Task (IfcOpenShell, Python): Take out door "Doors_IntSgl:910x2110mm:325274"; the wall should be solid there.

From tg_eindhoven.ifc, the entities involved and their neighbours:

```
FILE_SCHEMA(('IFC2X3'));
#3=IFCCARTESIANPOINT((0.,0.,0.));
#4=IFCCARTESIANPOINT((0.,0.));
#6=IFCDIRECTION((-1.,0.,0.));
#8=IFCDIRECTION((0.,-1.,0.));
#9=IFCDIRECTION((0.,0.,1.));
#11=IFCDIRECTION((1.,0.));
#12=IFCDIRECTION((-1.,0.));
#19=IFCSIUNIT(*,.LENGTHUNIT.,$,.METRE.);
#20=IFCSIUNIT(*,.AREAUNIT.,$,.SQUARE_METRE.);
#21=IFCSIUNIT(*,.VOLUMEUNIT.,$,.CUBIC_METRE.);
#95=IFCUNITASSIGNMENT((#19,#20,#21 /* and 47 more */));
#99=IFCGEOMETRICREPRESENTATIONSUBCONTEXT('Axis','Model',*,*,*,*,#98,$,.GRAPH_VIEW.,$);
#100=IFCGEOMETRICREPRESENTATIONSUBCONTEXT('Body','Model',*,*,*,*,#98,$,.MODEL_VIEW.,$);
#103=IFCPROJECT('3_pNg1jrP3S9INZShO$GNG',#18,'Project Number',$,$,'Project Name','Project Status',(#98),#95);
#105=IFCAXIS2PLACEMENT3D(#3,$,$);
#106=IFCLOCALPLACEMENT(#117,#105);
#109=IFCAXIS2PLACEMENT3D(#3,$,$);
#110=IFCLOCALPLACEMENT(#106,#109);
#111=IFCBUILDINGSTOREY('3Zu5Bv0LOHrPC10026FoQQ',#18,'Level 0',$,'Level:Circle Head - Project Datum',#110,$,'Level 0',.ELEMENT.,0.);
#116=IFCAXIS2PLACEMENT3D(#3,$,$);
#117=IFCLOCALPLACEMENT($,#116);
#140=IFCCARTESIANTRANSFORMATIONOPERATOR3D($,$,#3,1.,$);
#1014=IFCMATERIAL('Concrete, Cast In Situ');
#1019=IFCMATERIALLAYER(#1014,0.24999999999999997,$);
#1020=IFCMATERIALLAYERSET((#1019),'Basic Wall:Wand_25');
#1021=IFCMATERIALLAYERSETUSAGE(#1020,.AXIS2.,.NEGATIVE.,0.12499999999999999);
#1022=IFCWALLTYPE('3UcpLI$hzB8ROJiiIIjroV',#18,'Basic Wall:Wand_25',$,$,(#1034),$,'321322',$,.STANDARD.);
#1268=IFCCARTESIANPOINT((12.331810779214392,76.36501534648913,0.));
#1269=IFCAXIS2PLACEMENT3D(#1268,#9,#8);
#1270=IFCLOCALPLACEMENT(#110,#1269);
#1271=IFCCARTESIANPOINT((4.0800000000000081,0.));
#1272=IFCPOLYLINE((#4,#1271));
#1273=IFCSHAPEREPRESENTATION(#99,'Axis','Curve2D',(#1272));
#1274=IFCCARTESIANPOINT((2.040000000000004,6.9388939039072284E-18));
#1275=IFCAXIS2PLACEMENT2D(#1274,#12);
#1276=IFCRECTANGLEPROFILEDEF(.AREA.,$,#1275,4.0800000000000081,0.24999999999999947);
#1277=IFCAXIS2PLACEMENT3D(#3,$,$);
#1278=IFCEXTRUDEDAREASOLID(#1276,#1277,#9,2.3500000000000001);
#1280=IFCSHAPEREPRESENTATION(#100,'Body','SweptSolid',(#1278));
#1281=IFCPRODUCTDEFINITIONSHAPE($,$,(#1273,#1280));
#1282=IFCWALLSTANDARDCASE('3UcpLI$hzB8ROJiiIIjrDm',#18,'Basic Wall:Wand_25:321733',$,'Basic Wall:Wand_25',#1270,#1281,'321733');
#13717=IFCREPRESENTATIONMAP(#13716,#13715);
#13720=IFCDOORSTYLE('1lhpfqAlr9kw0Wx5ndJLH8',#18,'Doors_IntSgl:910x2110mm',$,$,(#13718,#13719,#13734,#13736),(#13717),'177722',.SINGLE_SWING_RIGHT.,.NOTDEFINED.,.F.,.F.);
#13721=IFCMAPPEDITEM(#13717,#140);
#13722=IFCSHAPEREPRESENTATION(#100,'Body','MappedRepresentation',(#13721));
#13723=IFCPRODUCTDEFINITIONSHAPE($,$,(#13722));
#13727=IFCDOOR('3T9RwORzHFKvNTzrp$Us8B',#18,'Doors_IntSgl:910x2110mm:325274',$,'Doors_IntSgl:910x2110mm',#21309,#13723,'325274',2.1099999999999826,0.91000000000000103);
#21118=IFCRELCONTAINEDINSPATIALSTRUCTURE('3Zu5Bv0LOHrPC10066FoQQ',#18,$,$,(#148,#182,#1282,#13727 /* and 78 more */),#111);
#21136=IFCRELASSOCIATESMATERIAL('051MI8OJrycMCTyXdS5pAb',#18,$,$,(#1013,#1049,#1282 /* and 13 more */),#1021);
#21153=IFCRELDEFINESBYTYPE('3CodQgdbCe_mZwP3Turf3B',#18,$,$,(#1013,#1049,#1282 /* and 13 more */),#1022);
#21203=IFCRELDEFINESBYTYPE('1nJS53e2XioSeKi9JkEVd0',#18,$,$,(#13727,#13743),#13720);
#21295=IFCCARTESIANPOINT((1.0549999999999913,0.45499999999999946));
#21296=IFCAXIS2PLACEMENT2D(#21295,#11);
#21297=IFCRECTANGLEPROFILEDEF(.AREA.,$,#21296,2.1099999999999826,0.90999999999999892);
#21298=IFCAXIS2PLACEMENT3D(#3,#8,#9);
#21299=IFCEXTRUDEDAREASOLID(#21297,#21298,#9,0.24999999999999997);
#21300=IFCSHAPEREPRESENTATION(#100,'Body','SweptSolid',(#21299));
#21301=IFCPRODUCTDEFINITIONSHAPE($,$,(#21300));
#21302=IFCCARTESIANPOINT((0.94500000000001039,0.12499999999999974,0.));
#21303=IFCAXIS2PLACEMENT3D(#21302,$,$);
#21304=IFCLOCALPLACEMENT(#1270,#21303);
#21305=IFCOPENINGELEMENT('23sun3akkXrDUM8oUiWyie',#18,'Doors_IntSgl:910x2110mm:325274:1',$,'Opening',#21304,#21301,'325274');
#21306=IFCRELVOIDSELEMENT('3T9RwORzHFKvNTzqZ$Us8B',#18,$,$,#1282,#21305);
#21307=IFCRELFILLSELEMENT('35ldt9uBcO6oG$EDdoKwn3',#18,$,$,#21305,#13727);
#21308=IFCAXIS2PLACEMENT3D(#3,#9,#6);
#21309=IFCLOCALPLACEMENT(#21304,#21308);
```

```python
import ifcopenshell
import ifcopenshell.api.feature
import ifcopenshell.api.root
import ifcopenshell.geom
import ifcopenshell.util.shape

model = ifcopenshell.open("tg_eindhoven.ifc")
settings = ifcopenshell.geom.settings()


def volume(element):
    """Net volume in cubic metres, openings subtracted."""
    shape = ifcopenshell.geom.create_shape(settings, element)
    return ifcopenshell.util.shape.get_volume(shape.geometry)


door = model.by_guid("3T9RwORzHFKvNTzrp$Us8B")
opening = door.FillsVoids[0].RelatingOpeningElement
wall = opening.VoidsElements[0].RelatingBuildingElement
before = volume(wall)

ifcopenshell.api.root.remove_product(model, product=door)
ifcopenshell.api.feature.remove_feature(model, feature=opening)

after = volume(wall)

print(f"wall volume {before:.3f} -> {after:.3f} m3")

model.write("tg_eindhoven_updated.ifc")
```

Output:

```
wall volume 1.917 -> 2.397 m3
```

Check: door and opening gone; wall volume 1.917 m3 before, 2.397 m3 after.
